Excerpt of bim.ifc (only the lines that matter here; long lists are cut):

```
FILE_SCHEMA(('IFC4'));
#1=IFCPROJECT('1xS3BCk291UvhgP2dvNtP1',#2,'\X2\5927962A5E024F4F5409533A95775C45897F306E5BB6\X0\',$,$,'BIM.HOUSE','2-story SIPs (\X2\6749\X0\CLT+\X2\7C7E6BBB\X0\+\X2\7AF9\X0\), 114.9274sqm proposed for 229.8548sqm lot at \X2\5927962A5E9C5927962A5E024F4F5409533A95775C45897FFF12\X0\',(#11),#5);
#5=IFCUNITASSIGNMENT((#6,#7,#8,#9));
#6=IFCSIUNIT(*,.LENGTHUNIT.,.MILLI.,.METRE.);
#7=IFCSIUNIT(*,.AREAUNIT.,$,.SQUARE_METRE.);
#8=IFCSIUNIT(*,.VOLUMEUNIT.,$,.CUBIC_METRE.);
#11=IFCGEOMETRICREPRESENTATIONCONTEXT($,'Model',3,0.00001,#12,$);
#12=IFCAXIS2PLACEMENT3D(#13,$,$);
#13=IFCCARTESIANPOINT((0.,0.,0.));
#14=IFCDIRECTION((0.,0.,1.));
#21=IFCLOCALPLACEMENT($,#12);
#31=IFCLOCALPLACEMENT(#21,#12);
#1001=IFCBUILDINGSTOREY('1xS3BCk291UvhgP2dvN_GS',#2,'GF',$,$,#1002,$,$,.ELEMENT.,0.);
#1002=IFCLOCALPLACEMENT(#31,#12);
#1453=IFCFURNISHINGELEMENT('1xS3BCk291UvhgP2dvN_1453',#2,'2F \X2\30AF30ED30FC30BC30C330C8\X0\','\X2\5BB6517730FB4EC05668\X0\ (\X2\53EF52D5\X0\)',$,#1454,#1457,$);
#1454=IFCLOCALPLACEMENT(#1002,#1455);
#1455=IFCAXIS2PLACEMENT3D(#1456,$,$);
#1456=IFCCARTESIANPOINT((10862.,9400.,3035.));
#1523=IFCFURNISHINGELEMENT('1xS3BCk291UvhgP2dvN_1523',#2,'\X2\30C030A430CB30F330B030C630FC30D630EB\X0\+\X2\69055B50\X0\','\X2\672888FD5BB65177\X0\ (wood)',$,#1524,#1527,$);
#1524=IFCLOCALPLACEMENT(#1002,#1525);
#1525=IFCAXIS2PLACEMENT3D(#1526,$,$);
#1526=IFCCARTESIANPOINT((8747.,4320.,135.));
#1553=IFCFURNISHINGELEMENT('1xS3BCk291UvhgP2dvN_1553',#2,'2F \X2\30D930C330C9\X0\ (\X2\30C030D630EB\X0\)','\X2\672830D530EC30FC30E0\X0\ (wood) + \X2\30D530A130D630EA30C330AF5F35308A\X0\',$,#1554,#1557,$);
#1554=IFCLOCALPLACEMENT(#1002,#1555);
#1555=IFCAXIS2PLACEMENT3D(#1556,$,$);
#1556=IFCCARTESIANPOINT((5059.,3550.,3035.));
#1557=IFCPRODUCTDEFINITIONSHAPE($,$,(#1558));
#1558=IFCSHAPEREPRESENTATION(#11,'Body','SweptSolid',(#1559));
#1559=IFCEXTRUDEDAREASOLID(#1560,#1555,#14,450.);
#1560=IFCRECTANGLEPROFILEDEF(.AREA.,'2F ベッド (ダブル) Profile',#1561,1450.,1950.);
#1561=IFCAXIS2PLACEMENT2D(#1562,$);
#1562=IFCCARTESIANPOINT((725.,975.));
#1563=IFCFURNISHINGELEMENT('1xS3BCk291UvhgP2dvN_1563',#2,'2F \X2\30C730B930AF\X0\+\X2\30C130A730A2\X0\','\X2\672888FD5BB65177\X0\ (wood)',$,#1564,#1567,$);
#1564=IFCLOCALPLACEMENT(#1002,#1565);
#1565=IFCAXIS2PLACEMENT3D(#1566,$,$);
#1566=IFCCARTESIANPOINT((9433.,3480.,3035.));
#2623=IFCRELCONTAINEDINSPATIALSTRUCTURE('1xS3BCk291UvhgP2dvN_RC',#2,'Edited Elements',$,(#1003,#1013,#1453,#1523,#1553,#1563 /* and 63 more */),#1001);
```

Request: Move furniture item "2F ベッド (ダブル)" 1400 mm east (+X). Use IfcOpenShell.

```python
import ifcopenshell
import ifcopenshell.api.geometry
import ifcopenshell.util.placement

model = ifcopenshell.open("bim.ifc")

item = model.by_guid("1xS3BCk291UvhgP2dvN_1553")
matrix = ifcopenshell.util.placement.get_local_placement(item.ObjectPlacement)
matrix[0, 3] += 1400.0
ifcopenshell.api.geometry.edit_object_placement(model, product=item, matrix=matrix, is_si=False)

print(ifcopenshell.util.placement.get_local_placement(item.ObjectPlacement).round(3) + 0.0)

model.write("bim_v2.ifc")
```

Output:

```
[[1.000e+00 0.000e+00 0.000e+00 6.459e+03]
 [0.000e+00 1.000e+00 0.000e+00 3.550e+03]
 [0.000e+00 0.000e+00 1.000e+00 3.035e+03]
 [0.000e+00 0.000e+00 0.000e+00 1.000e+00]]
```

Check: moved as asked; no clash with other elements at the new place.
